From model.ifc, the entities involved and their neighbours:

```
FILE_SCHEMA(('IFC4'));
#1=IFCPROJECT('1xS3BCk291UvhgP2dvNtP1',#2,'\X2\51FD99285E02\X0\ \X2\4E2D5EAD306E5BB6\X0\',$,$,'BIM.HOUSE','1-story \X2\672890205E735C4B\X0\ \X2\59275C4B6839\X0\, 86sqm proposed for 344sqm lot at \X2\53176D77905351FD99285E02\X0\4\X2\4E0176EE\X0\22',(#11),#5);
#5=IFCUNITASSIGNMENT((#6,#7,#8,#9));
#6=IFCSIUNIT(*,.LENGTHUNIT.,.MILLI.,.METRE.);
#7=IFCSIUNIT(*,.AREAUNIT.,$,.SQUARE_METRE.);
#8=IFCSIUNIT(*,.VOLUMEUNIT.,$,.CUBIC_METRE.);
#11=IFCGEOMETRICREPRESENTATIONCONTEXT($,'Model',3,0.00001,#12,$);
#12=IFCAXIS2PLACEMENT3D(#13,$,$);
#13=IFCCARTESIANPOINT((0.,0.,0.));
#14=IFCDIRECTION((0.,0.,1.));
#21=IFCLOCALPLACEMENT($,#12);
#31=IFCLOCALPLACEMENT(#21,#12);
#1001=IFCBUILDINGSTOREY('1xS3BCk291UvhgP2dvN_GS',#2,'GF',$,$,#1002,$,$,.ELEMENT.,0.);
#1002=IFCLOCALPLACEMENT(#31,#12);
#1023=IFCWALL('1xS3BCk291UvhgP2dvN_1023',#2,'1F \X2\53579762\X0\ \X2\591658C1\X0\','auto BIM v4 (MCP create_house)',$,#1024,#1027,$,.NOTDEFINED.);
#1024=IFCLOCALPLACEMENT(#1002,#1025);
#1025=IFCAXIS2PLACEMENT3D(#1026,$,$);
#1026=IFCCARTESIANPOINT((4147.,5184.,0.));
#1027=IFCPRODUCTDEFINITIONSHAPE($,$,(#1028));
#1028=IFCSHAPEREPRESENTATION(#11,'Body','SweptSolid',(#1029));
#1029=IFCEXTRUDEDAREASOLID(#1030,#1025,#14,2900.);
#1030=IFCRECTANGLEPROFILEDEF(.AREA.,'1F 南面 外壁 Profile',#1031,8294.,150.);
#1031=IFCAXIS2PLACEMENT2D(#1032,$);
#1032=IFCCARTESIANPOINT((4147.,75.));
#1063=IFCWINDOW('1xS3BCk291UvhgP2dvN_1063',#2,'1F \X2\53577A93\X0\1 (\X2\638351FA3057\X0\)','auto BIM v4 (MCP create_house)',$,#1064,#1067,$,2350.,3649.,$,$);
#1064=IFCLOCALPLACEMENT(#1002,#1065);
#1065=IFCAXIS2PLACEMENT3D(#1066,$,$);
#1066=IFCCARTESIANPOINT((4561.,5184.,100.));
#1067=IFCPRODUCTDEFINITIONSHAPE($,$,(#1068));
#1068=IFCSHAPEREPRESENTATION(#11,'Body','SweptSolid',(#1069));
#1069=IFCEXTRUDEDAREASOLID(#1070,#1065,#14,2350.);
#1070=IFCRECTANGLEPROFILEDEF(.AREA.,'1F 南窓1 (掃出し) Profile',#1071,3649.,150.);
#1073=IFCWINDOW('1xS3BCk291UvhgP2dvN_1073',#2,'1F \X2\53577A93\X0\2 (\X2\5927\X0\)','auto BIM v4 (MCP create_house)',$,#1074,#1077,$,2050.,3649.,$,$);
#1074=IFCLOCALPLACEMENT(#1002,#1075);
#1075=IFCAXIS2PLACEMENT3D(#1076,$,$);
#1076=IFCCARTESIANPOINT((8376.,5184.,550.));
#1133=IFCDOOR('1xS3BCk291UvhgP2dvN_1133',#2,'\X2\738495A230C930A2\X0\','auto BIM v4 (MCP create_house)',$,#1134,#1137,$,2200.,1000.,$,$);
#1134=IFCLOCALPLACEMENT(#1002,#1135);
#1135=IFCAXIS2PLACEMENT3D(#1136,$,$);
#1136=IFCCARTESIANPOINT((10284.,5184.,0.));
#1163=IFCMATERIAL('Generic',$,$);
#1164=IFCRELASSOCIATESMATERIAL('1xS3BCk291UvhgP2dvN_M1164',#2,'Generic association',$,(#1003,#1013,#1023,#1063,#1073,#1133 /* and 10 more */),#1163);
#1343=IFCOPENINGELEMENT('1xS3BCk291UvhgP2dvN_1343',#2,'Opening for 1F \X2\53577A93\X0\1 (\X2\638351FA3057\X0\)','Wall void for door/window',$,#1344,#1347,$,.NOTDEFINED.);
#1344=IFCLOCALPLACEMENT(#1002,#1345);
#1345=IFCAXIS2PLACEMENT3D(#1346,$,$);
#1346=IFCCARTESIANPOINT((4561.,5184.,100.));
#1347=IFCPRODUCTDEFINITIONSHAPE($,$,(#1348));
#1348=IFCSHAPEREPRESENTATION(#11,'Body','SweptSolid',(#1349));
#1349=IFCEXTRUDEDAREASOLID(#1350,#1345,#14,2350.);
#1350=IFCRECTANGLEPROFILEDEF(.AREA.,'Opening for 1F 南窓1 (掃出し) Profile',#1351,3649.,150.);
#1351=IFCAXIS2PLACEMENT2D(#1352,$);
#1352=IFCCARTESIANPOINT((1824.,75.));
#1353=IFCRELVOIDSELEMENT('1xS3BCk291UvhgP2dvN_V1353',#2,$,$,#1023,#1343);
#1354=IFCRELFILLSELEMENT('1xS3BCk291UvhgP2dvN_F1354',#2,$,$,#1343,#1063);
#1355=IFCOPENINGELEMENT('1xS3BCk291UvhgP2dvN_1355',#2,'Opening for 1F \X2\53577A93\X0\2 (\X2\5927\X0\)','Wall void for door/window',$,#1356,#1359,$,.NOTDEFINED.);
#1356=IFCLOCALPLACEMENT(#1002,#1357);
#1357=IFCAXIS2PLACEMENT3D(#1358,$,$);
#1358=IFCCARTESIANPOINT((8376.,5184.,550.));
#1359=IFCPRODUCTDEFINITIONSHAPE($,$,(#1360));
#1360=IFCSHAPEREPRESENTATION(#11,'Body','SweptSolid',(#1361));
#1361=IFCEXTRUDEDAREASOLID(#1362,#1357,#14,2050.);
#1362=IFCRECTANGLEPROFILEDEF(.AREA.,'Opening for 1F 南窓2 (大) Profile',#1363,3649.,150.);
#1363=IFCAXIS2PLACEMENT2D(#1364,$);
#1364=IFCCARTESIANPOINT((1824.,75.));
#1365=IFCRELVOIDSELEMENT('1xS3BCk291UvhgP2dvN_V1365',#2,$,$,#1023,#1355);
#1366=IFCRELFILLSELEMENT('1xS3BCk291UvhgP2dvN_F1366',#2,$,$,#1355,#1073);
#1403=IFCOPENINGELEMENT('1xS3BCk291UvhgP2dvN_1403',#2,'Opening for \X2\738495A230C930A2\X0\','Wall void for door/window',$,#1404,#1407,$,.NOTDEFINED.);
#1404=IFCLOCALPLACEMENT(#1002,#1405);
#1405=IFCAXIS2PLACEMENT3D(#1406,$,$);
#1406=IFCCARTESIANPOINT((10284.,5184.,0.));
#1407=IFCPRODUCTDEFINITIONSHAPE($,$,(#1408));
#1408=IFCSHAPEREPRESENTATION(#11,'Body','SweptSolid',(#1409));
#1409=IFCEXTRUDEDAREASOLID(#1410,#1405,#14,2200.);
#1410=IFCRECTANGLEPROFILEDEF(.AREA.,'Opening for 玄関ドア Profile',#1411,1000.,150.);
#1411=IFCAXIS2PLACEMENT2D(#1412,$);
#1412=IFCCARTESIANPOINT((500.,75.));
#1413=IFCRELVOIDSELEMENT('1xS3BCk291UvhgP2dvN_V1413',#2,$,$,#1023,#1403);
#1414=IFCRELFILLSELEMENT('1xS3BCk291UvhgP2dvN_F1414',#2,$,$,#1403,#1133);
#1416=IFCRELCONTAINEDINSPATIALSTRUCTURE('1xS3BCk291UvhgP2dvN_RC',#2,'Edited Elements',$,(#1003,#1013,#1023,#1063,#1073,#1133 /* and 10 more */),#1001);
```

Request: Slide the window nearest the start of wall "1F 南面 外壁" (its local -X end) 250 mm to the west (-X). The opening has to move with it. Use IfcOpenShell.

```python
import ifcopenshell
import ifcopenshell.api.geometry
import ifcopenshell.util.placement

model = ifcopenshell.open("model.ifc")

window = model.by_id(1063)
opening = window.FillsVoids[0].RelatingOpeningElement
wall = opening.VoidsElements[0].RelatingBuildingElement

wall_matrix = ifcopenshell.util.placement.get_local_placement(wall.ObjectPlacement)
shift = wall_matrix[:3, 0] * -250.0
before = ifcopenshell.util.placement.get_local_placement(window.ObjectPlacement)[:3, 3].copy()

# The window is not placed relative to its opening, so move both.
for product in (opening, window):
    matrix = ifcopenshell.util.placement.get_local_placement(product.ObjectPlacement)
    matrix[:3, 3] += shift
    ifcopenshell.api.geometry.edit_object_placement(model, product=product, matrix=matrix, is_si=False)

after = ifcopenshell.util.placement.get_local_placement(window.ObjectPlacement)[:3, 3]
print("window moved by", (after - before).round(3) + 0.0)

model.write("model_rev.ifc")
```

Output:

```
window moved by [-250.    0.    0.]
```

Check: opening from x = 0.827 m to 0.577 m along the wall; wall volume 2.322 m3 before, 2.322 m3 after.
